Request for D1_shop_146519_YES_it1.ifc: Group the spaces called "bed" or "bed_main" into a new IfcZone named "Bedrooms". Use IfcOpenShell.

First a look at what the model holds.

```python
import ifcopenshell

model = ifcopenshell.open("D1_shop_146519_YES_it1.ifc")
print(model.schema)
seen = {}
for space in model.by_type("IfcSpace"):
    seen[space.LongName] = seen.get(space.LongName, 0) + 1
for name, count in sorted(seen.items(), key=str):
    print(count, "x", name)
print("zones:", [z.Name for z in model.by_type("IfcZone")][:20])
```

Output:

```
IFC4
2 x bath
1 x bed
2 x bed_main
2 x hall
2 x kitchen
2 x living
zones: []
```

```python
import ifcopenshell
import ifcopenshell.api.group
import ifcopenshell.api.root

model = ifcopenshell.open("D1_shop_146519_YES_it1.ifc")

names = {"bed", "bed_main"}
spaces = [s for s in model.by_type("IfcSpace") if s.LongName in names]

zone = ifcopenshell.api.root.create_entity(model, ifc_class="IfcZone", name="Bedrooms")
ifcopenshell.api.group.assign_group(model, products=spaces, group=zone)
print(len(spaces), "spaces in", zone.Name)

model.write("D1_shop_146519_YES_it1_updated.ifc")
```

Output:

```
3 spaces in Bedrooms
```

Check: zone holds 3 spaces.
